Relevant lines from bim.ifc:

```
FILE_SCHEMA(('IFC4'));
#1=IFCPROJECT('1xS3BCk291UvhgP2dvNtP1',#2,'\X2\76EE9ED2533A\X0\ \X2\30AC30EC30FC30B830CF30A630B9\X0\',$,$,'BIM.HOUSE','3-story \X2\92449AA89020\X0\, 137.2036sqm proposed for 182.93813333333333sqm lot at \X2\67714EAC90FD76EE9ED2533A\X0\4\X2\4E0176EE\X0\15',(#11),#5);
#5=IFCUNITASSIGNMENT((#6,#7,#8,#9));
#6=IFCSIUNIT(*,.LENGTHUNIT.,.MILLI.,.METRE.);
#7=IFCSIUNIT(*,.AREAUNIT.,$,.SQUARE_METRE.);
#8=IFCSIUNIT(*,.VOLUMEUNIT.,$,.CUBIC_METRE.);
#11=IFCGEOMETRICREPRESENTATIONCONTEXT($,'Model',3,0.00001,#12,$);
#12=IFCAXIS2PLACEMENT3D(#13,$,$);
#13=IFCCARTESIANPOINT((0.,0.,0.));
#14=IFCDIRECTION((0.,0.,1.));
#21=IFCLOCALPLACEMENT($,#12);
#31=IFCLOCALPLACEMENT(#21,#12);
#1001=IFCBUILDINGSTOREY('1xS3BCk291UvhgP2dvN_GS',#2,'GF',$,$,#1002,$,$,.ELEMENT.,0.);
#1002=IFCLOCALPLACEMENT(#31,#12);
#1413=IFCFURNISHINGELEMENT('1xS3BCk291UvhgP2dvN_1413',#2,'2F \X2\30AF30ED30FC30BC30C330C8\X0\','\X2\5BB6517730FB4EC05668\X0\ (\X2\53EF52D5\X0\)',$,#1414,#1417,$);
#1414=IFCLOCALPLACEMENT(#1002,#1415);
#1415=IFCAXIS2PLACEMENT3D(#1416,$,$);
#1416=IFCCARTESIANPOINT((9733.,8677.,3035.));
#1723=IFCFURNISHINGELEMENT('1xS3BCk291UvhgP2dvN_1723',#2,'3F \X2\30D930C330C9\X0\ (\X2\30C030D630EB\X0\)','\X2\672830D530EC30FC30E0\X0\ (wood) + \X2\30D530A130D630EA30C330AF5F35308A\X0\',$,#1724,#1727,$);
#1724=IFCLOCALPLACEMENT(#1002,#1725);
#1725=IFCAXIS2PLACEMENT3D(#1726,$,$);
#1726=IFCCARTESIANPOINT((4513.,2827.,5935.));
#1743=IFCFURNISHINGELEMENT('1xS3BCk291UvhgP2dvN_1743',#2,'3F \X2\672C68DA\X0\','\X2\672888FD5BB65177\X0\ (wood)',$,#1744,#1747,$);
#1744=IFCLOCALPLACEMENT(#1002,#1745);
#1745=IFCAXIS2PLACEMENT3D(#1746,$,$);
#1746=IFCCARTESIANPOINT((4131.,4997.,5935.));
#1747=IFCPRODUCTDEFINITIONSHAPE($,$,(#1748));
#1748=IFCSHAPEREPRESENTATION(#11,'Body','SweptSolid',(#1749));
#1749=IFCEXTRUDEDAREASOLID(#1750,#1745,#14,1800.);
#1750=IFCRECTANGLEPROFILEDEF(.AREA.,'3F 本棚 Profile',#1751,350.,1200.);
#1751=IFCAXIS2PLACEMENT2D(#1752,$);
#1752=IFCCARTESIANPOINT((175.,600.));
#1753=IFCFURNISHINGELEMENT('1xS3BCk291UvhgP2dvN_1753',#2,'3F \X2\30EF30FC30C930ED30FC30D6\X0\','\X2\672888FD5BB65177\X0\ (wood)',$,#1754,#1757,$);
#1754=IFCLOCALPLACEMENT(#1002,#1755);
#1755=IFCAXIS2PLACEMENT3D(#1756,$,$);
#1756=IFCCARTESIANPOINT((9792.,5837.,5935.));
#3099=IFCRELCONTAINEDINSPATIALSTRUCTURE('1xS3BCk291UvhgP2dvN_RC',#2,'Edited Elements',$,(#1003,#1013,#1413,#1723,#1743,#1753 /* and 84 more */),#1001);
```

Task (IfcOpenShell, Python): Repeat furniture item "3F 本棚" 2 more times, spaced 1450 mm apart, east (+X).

```python
import numpy as np
import ifcopenshell
import ifcopenshell.api.geometry
import ifcopenshell.api.root
import ifcopenshell.util.element
import ifcopenshell.util.placement
import ifcopenshell.util.unit

model = ifcopenshell.open("bim.ifc")
unit_scale = ifcopenshell.util.unit.calculate_unit_scale(model)


def reuse_history(source, copy):
    """copy_class also copies each property set's owner history, people and application; keep the originals."""
    for rel in copy.IsDefinedBy:
        if rel.is_a("IfcRelDefinesByProperties") and (history := rel.RelatingPropertyDefinition.OwnerHistory):
            rel.RelatingPropertyDefinition.OwnerHistory = source.OwnerHistory
            ifcopenshell.util.element.remove_deep2(model, history)


source = model.by_guid("1xS3BCk291UvhgP2dvN_1743")
base = ifcopenshell.util.placement.get_local_placement(source.ObjectPlacement)
step = np.array([1.0, 0.0, 0.0]) * 1.45 / unit_scale

for i in range(1, 3):
    copy = ifcopenshell.api.root.copy_class(model, product=source)
    copy.Representation = ifcopenshell.util.element.copy_deep(
        model, source.Representation, exclude=["IfcGeometricRepresentationContext", "IfcRepresentationMap"]
    )
    reuse_history(source, copy)
    matrix = base.copy()
    matrix[:3, 3] += i * step
    print("added at", matrix[:3, 3].round(3) + 0.0)
    ifcopenshell.api.geometry.edit_object_placement(model, product=copy, matrix=matrix, is_si=False)

model.write("bim-out.ifc")
```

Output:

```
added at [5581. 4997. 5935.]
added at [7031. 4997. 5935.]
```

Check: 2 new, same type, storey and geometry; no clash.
